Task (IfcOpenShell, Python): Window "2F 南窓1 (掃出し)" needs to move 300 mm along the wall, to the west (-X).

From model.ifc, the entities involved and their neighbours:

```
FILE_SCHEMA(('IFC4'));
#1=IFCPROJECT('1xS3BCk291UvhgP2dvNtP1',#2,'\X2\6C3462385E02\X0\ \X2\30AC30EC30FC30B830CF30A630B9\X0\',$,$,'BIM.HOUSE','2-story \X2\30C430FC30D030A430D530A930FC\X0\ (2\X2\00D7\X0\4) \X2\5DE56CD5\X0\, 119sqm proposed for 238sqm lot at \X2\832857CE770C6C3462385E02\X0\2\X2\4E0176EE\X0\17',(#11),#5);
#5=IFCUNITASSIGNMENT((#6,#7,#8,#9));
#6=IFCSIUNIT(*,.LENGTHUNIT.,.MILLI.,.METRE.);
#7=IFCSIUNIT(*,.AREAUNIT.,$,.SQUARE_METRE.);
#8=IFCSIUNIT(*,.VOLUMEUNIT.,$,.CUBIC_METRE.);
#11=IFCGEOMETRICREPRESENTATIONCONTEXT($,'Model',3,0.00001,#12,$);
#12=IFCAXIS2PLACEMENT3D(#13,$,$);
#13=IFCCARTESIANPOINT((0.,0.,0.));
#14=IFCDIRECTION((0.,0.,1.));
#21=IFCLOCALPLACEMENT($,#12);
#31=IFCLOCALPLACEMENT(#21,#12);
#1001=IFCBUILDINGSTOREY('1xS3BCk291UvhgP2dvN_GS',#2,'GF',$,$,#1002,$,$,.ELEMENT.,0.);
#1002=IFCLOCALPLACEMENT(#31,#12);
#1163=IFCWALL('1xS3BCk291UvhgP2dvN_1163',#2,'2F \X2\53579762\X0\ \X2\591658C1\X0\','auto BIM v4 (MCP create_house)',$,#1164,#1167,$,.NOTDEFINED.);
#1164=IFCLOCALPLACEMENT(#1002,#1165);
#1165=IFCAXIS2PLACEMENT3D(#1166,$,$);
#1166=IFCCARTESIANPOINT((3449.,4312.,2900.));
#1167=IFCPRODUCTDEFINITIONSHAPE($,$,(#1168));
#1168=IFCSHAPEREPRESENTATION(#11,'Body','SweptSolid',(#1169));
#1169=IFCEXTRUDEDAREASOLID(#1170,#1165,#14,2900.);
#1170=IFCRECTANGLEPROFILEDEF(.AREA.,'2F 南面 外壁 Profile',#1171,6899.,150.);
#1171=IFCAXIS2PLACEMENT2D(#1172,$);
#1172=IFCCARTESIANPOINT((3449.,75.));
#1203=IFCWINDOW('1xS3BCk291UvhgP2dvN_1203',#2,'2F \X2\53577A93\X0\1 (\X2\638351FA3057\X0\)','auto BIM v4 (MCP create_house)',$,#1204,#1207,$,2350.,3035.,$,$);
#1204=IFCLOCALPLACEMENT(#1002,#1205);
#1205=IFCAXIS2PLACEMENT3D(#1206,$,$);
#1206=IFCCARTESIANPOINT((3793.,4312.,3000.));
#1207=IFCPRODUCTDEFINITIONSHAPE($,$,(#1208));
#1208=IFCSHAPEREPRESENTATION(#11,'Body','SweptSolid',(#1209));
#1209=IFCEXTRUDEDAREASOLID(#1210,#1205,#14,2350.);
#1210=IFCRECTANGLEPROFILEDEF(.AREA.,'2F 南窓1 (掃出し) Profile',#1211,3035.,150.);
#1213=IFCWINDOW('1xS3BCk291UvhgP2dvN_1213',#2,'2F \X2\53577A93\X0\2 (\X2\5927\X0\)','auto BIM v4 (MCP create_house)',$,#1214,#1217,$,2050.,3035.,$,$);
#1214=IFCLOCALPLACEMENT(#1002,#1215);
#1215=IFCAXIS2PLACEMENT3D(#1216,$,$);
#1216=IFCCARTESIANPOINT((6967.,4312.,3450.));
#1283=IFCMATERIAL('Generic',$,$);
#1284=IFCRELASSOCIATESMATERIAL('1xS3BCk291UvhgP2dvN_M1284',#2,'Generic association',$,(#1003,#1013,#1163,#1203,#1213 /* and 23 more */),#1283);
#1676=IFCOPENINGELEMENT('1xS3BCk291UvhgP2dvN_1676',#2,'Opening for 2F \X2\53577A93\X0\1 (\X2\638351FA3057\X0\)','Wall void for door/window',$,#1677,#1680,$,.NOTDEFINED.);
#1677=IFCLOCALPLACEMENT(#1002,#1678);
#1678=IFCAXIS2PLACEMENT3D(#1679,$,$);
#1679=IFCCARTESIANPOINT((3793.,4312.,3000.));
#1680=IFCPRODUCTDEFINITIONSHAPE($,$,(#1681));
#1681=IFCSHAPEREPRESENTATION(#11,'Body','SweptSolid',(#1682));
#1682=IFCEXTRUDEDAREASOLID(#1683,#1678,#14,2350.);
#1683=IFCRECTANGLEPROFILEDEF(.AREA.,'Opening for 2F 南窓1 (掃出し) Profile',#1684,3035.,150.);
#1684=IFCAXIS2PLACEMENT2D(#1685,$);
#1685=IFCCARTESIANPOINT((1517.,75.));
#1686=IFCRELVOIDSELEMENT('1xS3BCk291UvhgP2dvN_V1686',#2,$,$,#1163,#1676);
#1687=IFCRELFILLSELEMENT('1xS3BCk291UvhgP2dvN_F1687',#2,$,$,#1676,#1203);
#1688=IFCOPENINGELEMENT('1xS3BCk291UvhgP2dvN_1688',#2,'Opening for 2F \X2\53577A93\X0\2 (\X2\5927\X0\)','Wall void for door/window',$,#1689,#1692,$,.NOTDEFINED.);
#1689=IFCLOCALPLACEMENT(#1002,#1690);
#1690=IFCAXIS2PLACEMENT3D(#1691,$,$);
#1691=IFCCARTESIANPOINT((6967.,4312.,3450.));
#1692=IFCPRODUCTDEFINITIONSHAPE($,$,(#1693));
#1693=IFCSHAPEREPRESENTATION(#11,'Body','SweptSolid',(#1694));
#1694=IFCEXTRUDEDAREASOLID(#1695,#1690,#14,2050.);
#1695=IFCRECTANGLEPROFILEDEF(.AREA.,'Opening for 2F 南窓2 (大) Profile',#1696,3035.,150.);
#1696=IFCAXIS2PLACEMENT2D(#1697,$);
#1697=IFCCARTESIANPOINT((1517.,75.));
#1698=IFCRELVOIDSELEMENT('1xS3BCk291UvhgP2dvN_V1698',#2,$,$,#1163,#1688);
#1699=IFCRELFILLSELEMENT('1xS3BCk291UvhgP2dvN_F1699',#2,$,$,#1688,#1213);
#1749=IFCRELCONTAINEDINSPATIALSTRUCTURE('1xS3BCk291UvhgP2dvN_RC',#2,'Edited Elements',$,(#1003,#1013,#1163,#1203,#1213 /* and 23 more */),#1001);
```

```python
import ifcopenshell
import ifcopenshell.api.geometry
import ifcopenshell.util.placement
import ifcopenshell.util.unit

model = ifcopenshell.open("model.ifc")
unit_scale = ifcopenshell.util.unit.calculate_unit_scale(model)

window = model.by_guid("1xS3BCk291UvhgP2dvN_1203")
opening = window.FillsVoids[0].RelatingOpeningElement
wall = opening.VoidsElements[0].RelatingBuildingElement

wall_matrix = ifcopenshell.util.placement.get_local_placement(wall.ObjectPlacement)
shift = wall_matrix[:3, 0] * -0.3 / unit_scale
before = ifcopenshell.util.placement.get_local_placement(window.ObjectPlacement)[:3, 3].copy()

# The window is not placed relative to its opening, so move both.
for product in (opening, window):
    matrix = ifcopenshell.util.placement.get_local_placement(product.ObjectPlacement)
    matrix[:3, 3] += shift
    ifcopenshell.api.geometry.edit_object_placement(model, product=product, matrix=matrix, is_si=False)

after = ifcopenshell.util.placement.get_local_placement(window.ObjectPlacement)[:3, 3]
print("window moved by", (after - before).round(3) + 0.0)

model.write("model-out.ifc")
```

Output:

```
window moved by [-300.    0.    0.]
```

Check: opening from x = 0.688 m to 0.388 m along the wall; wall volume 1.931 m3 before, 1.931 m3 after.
